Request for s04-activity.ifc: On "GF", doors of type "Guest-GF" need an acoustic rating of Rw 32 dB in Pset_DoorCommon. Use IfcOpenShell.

First a look at what the model holds.

```python
import ifcopenshell
import ifcopenshell.util.element

model = ifcopenshell.open("s04-activity.ifc")
print(model.schema)
storey = next(s for s in model.by_type("IfcBuildingStorey") if s.Name == "GF")
doors = [e for e in ifcopenshell.util.element.get_decomposition(storey) if e.is_a("IfcDoor")]
seen = {}
for e in doors:
    element_type = ifcopenshell.util.element.get_type(e)
    key = (element_type.Name if element_type != e and element_type else None, ifcopenshell.util.element.get_pset(e, "Pset_DoorCommon", "AcousticRating"))
    seen[key] = seen.get(key, 0) + 1
for (name, value), count in sorted(seen.items(), key=str):
    print(count, "x", name, "|", value)
```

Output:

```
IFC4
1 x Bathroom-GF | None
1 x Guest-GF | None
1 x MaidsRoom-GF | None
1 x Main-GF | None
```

```python
import ifcopenshell
import ifcopenshell.api.pset
import ifcopenshell.util.element

model = ifcopenshell.open("s04-activity.ifc")

storey = next(s for s in model.by_type("IfcBuildingStorey") if s.Name == "GF")
doors = [e for e in ifcopenshell.util.element.get_decomposition(storey) if e.is_a("IfcDoor")]

count = 0
for e in doors:
    element_type = ifcopenshell.util.element.get_type(e)
    if element_type in (None, e) or element_type.Name != "Guest-GF":
        continue
    # add_pset returns the element's existing set when there is one.
    pset = ifcopenshell.api.pset.add_pset(model, product=e, name="Pset_DoorCommon")
    ifcopenshell.api.pset.edit_pset(model, pset=pset, properties={"AcousticRating": "Rw 32 dB"})
    count += 1

print(count, "doors updated")

model.write("s04-activity_updated.ifc")
```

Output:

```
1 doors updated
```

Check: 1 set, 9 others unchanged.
